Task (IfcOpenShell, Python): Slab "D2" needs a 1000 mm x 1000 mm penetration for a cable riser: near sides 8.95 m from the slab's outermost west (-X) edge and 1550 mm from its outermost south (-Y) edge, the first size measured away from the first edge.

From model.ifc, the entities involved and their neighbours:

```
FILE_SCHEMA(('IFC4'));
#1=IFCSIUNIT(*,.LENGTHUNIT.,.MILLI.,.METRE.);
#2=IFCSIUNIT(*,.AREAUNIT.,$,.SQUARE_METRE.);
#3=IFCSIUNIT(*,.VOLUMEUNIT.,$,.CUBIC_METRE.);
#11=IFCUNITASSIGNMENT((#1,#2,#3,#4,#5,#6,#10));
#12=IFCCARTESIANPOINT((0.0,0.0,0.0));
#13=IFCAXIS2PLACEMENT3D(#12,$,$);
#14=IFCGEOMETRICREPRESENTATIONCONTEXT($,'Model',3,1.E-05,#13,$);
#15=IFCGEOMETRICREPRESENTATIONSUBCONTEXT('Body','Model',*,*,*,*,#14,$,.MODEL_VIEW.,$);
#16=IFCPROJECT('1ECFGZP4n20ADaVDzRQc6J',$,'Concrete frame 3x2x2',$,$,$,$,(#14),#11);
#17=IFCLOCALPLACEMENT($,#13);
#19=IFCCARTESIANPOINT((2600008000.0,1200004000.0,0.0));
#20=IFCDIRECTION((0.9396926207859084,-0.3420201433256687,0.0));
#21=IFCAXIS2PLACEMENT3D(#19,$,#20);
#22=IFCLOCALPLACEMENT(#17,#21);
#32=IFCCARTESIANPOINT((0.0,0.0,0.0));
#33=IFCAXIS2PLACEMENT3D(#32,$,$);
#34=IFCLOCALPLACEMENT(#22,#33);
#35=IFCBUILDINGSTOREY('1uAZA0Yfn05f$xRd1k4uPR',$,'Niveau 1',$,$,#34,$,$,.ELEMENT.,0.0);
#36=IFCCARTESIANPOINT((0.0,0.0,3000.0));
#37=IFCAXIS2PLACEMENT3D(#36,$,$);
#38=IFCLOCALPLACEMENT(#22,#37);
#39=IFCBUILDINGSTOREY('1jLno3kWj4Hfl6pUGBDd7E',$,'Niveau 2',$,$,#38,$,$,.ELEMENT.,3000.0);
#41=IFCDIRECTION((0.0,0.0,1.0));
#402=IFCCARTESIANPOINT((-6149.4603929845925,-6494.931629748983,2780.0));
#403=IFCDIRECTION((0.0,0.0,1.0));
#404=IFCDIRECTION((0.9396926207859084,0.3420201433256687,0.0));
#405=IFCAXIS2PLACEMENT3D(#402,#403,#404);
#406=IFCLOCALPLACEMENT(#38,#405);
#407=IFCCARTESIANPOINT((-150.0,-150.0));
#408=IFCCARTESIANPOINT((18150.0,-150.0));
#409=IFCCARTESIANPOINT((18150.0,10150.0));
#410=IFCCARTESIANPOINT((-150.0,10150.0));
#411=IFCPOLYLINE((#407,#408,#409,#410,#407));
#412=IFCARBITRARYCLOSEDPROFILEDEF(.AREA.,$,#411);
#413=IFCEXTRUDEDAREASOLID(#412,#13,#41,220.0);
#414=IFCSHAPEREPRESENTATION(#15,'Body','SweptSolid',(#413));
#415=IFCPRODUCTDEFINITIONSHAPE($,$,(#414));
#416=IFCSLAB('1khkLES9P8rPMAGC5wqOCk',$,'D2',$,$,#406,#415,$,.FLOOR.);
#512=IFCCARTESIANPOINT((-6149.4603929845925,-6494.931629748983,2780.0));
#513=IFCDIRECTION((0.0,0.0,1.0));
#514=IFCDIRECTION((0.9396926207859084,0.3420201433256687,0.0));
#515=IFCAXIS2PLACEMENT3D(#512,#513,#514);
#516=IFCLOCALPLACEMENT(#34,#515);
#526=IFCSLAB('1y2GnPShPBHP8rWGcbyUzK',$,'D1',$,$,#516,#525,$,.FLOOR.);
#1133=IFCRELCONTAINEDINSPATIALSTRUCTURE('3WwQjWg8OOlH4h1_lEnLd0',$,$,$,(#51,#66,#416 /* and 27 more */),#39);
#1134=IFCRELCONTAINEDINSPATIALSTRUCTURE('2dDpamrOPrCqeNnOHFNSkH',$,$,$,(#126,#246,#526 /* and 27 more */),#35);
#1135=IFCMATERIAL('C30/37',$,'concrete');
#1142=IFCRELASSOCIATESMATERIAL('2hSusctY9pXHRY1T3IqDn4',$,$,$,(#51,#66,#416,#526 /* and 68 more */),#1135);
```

```python
import numpy as np
import ifcopenshell
import ifcopenshell.api.feature
import ifcopenshell.api.geometry
import ifcopenshell.api.root
import ifcopenshell.geom
import ifcopenshell.util.placement
import ifcopenshell.util.representation
import ifcopenshell.util.shape
import ifcopenshell.util.unit

model = ifcopenshell.open("model.ifc")
unit_scale = ifcopenshell.util.unit.calculate_unit_scale(model)
settings = ifcopenshell.geom.settings()


def volume(element):
    """Net volume in cubic metres, openings subtracted."""
    shape = ifcopenshell.geom.create_shape(settings, element)
    return ifcopenshell.util.shape.get_volume(shape.geometry)


slab = model.by_guid("1khkLES9P8rPMAGC5wqOCk")
before = volume(slab)

# Extent in the slab's own axes, in metres. The edges named are its -X and -Y sides.
slab_shape = ifcopenshell.geom.create_shape(settings, slab)
vertices = ifcopenshell.util.shape.get_vertices(slab_shape.geometry)
x_min, y_min, bottom = vertices.min(axis=0)
top = vertices[:, 2].max()

opening = ifcopenshell.api.root.create_entity(model, ifc_class="IfcOpeningElement", name="Cable riser opening", predefined_type="OPENING")
context = ifcopenshell.util.representation.get_context(model, "Model", "Body", "MODEL_VIEW")
width, depth = 1, 1
outline = [(0.0, 0.0), (width, 0.0), (width, depth), (0.0, depth), (0.0, 0.0)]
# Overshoot both faces by 50 mm so the cut is clean.
shape = ifcopenshell.api.geometry.add_slab_representation(
    model, context=context, depth=top - bottom + 0.1, polyline=outline
)
ifcopenshell.api.geometry.assign_representation(model, product=opening, representation=shape)

matrix = ifcopenshell.util.placement.get_local_placement(slab.ObjectPlacement)
matrix[:, 3] = matrix @ np.append(np.array([x_min + 8.95, y_min + 1.55, bottom - 0.05]) / unit_scale, 1.0)
ifcopenshell.api.geometry.edit_object_placement(model, product=opening, matrix=matrix, is_si=False)
ifcopenshell.api.feature.add_feature(model, feature=opening, element=slab)

after = volume(slab)

print(f"slab volume {before:.3f} -> {after:.3f} m3")

model.write("model_v2.ifc")
```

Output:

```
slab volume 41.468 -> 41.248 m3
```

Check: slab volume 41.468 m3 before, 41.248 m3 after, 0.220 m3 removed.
